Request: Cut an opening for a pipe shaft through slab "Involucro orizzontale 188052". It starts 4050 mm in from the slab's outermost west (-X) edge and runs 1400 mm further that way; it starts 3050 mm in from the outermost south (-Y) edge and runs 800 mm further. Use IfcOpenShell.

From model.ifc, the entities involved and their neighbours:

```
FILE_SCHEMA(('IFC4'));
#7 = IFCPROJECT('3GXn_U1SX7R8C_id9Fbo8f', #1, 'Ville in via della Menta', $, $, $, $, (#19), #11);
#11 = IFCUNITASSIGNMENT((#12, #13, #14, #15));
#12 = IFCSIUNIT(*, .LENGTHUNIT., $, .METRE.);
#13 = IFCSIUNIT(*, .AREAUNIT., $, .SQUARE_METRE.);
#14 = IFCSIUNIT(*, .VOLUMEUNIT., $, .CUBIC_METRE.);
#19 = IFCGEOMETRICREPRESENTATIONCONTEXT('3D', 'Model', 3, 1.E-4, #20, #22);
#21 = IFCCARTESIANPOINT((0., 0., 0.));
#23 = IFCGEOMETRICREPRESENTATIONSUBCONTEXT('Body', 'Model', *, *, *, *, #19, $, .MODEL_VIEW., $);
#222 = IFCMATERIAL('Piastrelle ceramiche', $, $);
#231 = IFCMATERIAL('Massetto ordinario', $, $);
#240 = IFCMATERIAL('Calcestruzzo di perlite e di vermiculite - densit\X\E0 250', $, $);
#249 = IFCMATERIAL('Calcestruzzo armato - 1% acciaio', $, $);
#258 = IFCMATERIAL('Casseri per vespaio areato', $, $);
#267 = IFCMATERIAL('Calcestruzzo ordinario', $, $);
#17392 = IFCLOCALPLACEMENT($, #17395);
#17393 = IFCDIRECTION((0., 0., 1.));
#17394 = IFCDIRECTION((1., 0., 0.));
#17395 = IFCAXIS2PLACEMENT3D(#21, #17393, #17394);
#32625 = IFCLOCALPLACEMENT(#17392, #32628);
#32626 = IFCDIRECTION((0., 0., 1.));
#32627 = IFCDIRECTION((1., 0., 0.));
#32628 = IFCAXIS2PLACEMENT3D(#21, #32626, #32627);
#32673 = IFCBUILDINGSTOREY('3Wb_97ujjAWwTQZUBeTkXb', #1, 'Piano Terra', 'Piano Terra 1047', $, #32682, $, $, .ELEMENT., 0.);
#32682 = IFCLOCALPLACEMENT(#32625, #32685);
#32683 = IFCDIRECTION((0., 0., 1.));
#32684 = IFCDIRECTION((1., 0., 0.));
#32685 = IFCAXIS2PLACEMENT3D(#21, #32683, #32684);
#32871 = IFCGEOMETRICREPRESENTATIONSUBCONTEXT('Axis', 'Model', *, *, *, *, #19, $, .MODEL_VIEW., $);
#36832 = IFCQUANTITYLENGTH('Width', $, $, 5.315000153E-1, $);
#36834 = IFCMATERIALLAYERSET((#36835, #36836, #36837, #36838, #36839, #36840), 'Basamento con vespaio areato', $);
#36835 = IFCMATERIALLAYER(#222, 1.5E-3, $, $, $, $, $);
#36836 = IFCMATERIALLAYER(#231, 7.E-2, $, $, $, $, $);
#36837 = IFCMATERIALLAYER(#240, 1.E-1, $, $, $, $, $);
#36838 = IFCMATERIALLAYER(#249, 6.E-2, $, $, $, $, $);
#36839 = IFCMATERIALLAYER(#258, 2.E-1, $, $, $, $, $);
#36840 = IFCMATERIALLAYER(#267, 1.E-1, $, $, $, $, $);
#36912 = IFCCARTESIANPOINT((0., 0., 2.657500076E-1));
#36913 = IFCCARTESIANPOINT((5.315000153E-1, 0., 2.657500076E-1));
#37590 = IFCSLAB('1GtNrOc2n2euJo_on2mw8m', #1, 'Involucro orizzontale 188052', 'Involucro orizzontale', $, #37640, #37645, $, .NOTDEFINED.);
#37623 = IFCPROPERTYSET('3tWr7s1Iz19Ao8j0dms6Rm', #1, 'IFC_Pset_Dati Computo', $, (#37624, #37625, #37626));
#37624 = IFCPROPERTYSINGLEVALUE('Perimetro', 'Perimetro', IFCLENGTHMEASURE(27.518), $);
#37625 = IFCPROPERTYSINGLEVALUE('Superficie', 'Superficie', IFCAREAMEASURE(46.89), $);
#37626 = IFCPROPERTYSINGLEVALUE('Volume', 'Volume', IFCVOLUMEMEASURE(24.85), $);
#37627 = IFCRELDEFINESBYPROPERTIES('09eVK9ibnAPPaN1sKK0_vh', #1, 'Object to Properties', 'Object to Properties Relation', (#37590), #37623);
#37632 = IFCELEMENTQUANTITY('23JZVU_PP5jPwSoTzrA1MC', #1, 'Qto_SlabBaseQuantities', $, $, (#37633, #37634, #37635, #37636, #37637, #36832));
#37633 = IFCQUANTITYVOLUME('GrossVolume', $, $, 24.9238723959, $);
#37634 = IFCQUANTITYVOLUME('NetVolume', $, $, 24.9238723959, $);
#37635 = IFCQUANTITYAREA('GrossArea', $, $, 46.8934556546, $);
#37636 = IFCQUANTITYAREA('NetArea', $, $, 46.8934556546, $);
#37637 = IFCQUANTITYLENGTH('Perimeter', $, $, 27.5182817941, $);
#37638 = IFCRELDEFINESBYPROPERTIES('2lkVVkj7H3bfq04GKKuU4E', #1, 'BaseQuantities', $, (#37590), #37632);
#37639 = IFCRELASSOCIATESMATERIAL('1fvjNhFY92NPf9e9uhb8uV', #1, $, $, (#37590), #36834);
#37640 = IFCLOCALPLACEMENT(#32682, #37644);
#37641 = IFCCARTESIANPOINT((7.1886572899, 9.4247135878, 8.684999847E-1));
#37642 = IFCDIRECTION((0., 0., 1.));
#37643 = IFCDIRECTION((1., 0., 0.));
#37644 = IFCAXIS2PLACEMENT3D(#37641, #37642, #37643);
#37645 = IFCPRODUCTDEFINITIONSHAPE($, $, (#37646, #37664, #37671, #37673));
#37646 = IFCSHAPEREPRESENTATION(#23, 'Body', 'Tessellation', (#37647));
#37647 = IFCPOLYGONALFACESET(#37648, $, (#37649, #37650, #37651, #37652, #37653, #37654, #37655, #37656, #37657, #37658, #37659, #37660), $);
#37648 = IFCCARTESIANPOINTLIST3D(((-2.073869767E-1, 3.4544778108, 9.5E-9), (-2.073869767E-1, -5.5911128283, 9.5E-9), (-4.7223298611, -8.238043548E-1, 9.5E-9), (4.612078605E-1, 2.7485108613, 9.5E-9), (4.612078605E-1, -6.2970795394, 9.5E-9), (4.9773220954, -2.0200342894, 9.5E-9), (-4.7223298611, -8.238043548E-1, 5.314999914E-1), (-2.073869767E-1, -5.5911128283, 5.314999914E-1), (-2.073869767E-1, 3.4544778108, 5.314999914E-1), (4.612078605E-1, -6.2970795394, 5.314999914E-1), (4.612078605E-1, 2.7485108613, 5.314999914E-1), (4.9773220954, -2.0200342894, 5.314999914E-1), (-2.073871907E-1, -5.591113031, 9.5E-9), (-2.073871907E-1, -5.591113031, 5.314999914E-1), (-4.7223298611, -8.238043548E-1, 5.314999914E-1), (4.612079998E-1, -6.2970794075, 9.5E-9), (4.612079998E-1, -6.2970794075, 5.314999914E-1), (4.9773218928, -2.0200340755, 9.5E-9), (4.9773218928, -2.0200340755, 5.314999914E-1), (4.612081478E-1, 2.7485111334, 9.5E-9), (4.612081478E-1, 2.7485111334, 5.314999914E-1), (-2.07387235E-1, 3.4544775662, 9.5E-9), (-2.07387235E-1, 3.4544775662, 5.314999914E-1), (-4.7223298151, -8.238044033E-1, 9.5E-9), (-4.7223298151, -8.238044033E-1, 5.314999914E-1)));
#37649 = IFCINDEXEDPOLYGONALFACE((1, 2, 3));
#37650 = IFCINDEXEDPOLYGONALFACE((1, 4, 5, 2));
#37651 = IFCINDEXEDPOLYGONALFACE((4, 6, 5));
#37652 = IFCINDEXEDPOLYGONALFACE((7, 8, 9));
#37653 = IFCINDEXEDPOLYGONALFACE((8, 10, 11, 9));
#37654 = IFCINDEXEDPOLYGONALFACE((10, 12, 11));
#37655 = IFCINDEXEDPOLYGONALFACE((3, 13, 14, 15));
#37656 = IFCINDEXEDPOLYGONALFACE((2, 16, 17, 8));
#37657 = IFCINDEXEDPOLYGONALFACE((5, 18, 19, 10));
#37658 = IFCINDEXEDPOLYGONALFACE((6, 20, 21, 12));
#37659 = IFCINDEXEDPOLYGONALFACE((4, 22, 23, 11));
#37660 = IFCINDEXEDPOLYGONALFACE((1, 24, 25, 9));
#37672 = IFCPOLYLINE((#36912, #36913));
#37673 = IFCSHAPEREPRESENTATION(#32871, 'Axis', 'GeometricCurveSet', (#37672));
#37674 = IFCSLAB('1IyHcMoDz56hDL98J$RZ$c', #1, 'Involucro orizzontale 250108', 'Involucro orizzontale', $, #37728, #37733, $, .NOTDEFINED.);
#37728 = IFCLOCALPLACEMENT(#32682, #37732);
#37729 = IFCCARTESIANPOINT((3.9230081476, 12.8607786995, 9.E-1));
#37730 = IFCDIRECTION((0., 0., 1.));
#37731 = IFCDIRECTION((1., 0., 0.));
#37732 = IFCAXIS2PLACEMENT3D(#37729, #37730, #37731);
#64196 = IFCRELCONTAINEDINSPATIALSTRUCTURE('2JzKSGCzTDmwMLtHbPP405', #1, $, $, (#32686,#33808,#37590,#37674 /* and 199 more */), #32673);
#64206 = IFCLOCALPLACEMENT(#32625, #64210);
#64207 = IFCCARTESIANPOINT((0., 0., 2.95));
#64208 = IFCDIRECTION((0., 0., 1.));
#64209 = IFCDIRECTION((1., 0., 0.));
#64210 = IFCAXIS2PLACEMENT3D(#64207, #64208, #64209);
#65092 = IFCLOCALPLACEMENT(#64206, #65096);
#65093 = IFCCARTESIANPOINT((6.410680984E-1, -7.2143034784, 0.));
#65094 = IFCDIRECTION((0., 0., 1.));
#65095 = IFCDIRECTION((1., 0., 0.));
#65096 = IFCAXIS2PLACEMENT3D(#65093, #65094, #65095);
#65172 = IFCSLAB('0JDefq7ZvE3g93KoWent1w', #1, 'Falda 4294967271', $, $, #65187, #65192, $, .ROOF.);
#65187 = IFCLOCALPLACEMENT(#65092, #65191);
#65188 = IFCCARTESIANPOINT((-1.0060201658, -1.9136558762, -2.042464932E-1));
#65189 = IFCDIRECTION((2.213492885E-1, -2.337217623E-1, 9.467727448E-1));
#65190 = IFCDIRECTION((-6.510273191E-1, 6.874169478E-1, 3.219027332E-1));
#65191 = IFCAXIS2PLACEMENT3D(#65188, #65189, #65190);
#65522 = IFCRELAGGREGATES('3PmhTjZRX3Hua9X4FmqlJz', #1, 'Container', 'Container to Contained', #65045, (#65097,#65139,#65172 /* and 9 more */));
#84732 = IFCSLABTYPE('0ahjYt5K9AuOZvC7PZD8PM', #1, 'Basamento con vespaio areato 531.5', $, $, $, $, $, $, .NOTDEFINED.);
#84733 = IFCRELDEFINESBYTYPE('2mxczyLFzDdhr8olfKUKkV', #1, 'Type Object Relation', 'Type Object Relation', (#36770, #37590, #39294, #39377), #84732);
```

```python
import numpy as np
import ifcopenshell
import ifcopenshell.api.feature
import ifcopenshell.api.geometry
import ifcopenshell.api.pset
import ifcopenshell.api.root
import ifcopenshell.geom
import ifcopenshell.util.element
import ifcopenshell.util.placement
import ifcopenshell.util.representation
import ifcopenshell.util.shape
import ifcopenshell.util.unit

model = ifcopenshell.open("model.ifc")
unit_scale = ifcopenshell.util.unit.calculate_unit_scale(model)
area_scale = ifcopenshell.util.unit.calculate_unit_scale(model, "AREAUNIT")
volume_scale = ifcopenshell.util.unit.calculate_unit_scale(model, "VOLUMEUNIT")
settings = ifcopenshell.geom.settings()


def volume(element):
    """Net volume in cubic metres, openings subtracted."""
    shape = ifcopenshell.geom.create_shape(settings, element)
    return ifcopenshell.util.shape.get_volume(shape.geometry)


slab = model.by_id(37590)
before = volume(slab)

# Extent in the slab's own axes, in metres. The edges named are its -X and -Y sides.
slab_shape = ifcopenshell.geom.create_shape(settings, slab)
vertices = ifcopenshell.util.shape.get_vertices(slab_shape.geometry)
x_min, y_min, bottom = vertices.min(axis=0)
top = vertices[:, 2].max()

opening = ifcopenshell.api.root.create_entity(model, ifc_class="IfcOpeningElement", name="Pipe shaft opening", predefined_type="OPENING")
context = ifcopenshell.util.representation.get_context(model, "Model", "Body", "MODEL_VIEW")
width, depth = 1.4, 0.8
outline = [(0.0, 0.0), (width, 0.0), (width, depth), (0.0, depth), (0.0, 0.0)]
# Overshoot both faces by 50 mm so the cut is clean.
shape = ifcopenshell.api.geometry.add_slab_representation(
    model, context=context, depth=top - bottom + 0.1, polyline=outline
)
ifcopenshell.api.geometry.assign_representation(model, product=opening, representation=shape)

matrix = ifcopenshell.util.placement.get_local_placement(slab.ObjectPlacement)
matrix[:, 3] = matrix @ np.append(np.array([x_min + 4.05, y_min + 3.05, bottom - 0.05]) / unit_scale, 1.0)
ifcopenshell.api.geometry.edit_object_placement(model, product=opening, matrix=matrix, is_si=False)
ifcopenshell.api.feature.add_feature(model, feature=opening, element=slab)

after = volume(slab)

# Update the slab's stored quantities.
pset = model.by_id(ifcopenshell.util.element.get_pset(slab, "IFC_Pset_Dati Computo", should_inherit=False)["id"])
ifcopenshell.api.pset.edit_pset(model, pset=pset, properties={
    "Superficie": model.create_entity("IfcAreaMeasure", after / (top - bottom) / area_scale),
    "Volume": model.create_entity("IfcVolumeMeasure", after / volume_scale),
})
qto = model.by_id(ifcopenshell.util.element.get_pset(slab, "Qto_SlabBaseQuantities", should_inherit=False)["id"])
ifcopenshell.api.pset.edit_qto(model, qto=qto, properties={
    "NetVolume": after / volume_scale,
    "NetArea": after / (top - bottom) / area_scale,
})

print(f"slab volume {before:.3f} -> {after:.3f} m3")

model.write("model_rev.ifc")
```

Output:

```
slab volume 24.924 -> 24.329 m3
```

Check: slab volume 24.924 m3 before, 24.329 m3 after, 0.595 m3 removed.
